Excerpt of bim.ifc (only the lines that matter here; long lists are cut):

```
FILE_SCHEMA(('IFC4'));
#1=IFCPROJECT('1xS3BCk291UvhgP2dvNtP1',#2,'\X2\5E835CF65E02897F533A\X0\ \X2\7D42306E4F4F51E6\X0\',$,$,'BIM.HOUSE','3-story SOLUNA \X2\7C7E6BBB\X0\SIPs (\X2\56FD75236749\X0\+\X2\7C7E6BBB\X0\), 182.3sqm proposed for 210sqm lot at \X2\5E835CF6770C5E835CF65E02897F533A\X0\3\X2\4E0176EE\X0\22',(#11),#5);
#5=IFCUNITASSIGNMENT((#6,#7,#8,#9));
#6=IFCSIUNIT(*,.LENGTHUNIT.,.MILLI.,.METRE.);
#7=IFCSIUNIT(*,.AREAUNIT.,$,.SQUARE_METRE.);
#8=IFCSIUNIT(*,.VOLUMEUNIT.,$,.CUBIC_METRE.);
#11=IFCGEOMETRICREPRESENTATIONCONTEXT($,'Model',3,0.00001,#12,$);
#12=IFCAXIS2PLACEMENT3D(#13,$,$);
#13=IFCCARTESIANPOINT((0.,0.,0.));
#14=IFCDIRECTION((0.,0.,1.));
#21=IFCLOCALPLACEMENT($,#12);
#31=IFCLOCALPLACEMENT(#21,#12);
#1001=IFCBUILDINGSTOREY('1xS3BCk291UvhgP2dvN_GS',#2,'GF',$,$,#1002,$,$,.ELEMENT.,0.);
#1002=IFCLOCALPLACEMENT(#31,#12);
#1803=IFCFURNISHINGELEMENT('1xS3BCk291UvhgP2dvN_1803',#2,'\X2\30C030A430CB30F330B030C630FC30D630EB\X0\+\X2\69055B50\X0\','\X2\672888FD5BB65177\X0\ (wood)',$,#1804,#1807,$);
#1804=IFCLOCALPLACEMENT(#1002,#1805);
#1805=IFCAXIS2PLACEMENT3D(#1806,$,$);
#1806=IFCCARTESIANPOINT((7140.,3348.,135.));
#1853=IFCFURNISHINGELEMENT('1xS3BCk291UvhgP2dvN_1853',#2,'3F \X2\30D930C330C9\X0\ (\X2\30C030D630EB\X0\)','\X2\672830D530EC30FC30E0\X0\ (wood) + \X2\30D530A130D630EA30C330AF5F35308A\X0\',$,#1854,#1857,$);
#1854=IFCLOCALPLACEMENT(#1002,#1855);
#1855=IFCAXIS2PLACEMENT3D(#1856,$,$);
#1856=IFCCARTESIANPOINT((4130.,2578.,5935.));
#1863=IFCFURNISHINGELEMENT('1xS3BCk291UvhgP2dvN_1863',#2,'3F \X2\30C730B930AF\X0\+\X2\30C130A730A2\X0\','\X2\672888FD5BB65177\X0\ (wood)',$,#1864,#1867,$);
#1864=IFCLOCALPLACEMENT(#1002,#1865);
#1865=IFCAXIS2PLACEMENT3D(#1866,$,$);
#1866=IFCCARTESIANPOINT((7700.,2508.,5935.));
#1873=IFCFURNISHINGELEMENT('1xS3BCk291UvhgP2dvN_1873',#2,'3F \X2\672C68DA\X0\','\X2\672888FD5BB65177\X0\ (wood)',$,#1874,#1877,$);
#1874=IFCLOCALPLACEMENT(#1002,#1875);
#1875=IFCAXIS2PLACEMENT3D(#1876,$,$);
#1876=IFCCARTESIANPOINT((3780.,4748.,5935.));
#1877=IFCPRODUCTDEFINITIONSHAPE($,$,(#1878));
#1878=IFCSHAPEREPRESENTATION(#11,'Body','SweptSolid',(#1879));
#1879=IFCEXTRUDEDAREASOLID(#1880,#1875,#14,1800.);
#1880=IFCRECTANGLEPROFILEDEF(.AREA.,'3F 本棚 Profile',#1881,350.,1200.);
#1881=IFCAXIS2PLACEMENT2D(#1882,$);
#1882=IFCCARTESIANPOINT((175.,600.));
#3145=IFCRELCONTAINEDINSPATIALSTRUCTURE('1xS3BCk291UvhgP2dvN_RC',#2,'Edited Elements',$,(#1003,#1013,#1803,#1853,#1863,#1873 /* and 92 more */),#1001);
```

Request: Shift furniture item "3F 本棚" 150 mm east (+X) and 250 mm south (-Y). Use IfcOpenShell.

```python
import ifcopenshell
import ifcopenshell.api.geometry
import ifcopenshell.util.placement
import ifcopenshell.util.unit

model = ifcopenshell.open("bim.ifc")
unit_scale = ifcopenshell.util.unit.calculate_unit_scale(model)

item = model.by_guid("1xS3BCk291UvhgP2dvN_1873")
matrix = ifcopenshell.util.placement.get_local_placement(item.ObjectPlacement)
matrix[0, 3] += 0.15 / unit_scale
matrix[1, 3] -= 0.25 / unit_scale
ifcopenshell.api.geometry.edit_object_placement(model, product=item, matrix=matrix, is_si=False)

print(ifcopenshell.util.placement.get_local_placement(item.ObjectPlacement).round(3) + 0.0)

model.write("bim_edited.ifc")
```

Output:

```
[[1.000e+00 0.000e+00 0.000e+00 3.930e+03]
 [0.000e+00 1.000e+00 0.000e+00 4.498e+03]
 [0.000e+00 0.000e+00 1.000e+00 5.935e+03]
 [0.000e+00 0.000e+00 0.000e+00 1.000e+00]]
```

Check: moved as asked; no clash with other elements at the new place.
